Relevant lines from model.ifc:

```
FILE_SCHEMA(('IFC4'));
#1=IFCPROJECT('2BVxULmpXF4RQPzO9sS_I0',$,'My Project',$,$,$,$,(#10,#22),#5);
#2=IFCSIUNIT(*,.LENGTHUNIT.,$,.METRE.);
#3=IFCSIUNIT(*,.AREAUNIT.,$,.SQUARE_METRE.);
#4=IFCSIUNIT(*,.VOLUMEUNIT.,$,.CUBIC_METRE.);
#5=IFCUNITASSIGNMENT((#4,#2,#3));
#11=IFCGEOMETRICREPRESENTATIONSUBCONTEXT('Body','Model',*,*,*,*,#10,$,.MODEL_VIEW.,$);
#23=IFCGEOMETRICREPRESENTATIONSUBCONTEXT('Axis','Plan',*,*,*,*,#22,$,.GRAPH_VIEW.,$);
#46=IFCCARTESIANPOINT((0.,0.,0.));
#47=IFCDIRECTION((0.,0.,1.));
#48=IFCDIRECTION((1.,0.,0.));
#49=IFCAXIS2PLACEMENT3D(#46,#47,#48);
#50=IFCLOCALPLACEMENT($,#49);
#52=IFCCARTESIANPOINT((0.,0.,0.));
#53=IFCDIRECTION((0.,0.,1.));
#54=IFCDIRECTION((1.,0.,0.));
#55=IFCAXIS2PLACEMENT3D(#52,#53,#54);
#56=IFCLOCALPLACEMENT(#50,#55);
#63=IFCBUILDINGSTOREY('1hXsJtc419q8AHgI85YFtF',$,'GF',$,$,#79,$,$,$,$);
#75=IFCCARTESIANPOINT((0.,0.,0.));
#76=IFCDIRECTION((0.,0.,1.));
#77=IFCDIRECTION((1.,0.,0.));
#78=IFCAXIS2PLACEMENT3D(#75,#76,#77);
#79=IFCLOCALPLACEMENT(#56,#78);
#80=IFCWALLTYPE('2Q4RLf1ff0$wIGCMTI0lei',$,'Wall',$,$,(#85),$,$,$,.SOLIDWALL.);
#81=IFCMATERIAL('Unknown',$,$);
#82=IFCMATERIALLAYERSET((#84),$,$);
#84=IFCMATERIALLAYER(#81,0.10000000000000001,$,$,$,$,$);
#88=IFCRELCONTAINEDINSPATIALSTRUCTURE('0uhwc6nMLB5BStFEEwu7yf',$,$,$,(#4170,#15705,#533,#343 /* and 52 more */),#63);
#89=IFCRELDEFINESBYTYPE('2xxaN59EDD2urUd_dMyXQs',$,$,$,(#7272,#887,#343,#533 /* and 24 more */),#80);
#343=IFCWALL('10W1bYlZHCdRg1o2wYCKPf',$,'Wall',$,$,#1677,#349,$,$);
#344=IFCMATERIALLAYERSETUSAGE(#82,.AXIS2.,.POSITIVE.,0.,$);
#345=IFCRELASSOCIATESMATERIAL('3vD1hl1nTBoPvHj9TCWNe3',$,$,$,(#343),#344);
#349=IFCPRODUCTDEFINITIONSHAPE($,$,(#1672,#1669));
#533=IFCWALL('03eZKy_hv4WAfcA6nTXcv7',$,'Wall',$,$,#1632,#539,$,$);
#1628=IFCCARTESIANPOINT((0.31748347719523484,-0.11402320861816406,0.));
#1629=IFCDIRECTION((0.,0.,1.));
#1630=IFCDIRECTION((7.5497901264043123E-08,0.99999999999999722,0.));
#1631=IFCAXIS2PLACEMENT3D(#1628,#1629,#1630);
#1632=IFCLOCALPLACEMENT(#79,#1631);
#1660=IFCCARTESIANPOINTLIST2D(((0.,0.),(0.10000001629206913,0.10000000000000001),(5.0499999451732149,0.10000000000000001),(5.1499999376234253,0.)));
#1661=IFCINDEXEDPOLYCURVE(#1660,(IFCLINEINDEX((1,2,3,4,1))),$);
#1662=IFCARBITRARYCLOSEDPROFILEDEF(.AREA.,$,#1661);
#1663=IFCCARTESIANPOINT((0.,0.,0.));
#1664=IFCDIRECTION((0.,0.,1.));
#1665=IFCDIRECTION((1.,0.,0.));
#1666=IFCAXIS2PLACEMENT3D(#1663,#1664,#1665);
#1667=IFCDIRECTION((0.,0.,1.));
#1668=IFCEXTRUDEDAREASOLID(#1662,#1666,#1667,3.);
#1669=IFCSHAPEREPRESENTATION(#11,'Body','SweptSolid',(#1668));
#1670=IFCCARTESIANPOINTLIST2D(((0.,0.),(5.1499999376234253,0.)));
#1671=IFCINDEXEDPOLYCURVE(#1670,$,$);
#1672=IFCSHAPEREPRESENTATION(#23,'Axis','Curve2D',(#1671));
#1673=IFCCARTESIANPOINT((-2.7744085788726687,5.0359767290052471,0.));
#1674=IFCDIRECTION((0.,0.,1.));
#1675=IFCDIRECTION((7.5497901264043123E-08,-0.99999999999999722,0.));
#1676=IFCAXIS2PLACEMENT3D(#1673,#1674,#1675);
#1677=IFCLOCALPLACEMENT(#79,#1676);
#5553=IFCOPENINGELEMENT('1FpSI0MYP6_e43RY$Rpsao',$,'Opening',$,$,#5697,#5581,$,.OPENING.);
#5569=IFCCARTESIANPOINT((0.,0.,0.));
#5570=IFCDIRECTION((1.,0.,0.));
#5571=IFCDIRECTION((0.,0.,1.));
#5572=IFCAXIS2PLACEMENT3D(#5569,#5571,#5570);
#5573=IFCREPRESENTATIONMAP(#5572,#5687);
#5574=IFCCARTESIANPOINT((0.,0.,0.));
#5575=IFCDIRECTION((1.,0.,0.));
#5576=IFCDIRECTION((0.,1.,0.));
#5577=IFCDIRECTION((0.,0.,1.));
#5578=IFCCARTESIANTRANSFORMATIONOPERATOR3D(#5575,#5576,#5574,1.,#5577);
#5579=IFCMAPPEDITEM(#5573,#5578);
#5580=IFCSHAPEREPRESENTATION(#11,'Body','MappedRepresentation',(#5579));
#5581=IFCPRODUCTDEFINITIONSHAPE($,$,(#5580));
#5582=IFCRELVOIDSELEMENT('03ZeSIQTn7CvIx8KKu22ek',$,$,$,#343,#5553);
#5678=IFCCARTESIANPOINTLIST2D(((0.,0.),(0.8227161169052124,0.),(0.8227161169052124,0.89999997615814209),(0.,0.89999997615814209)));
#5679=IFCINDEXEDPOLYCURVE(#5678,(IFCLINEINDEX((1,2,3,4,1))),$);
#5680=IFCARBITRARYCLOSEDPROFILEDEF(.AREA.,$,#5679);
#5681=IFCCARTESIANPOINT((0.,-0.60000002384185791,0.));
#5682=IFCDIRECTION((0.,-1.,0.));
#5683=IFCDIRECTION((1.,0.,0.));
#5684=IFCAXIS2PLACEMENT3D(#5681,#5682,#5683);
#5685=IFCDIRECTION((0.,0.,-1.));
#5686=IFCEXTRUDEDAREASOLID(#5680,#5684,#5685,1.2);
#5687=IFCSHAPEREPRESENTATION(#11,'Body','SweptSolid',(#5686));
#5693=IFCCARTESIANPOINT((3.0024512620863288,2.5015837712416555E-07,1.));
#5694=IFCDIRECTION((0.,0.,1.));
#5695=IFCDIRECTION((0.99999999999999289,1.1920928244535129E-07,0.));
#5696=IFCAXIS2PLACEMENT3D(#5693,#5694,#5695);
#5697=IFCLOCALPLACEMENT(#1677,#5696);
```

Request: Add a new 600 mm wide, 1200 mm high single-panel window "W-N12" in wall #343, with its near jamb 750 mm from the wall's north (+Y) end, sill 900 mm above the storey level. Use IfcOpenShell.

```python
import numpy as np
import ifcopenshell
import ifcopenshell.api.feature
import ifcopenshell.api.geometry
import ifcopenshell.api.root
import ifcopenshell.api.spatial
import ifcopenshell.geom
import ifcopenshell.util.element
import ifcopenshell.util.placement
import ifcopenshell.util.representation
import ifcopenshell.util.shape
import ifcopenshell.util.unit

model = ifcopenshell.open("model.ifc")
unit_scale = ifcopenshell.util.unit.calculate_unit_scale(model)
settings = ifcopenshell.geom.settings()


def volume(element):
    """Net volume in cubic metres, openings subtracted."""
    shape = ifcopenshell.geom.create_shape(settings, element)
    return ifcopenshell.util.shape.get_volume(shape.geometry)


wall = model.by_guid("10W1bYlZHCdRg1o2wYCKPf")
storey = ifcopenshell.util.element.get_container(wall, ifc_class="IfcBuildingStorey")
context = ifcopenshell.util.representation.get_context(model, "Model", "Body", "MODEL_VIEW")
before = volume(wall)

width, height, from_end, sill = 0.6, 1.2, 0.75, 0.9  # metres

# The wall runs along its own X axis, and the end named is its -X end.
wall_shape = ifcopenshell.geom.create_shape(settings, wall)
x, y, z = ifcopenshell.util.shape.get_vertices(wall_shape.geometry).T
start = x.min() + from_end
face, thickness = float(y.min()), float(y.max() - y.min())
wall_matrix = ifcopenshell.util.placement.get_local_placement(wall.ObjectPlacement)
level = ifcopenshell.util.placement.get_local_placement(storey.ObjectPlacement)[2, 3]


def in_wall(x, y):
    """Placement at x, y metres in the wall's axes, at sill height."""
    matrix = wall_matrix.copy()
    matrix[:, 3] = wall_matrix @ np.array([x / unit_scale, y / unit_scale, 0.0, 1.0])
    matrix[2, 3] = level + sill / unit_scale
    return matrix


# Opening: a box that overshoots both wall faces by 50 mm.
opening = ifcopenshell.api.root.create_entity(model, ifc_class="IfcOpeningElement", predefined_type="OPENING")
box = ifcopenshell.api.geometry.add_wall_representation(
    model, context=context, length=width, height=height, thickness=thickness + 0.1
)
ifcopenshell.api.geometry.assign_representation(model, product=opening, representation=box)
ifcopenshell.api.geometry.edit_object_placement(model, product=opening, matrix=in_wall(start, face - 0.05), is_si=False)
ifcopenshell.api.feature.add_feature(model, feature=opening, element=wall)

window = ifcopenshell.api.root.create_entity(model, ifc_class="IfcWindow", name="W-N12", predefined_type="WINDOW")
window.OverallWidth, window.OverallHeight = width / unit_scale, height / unit_scale
window.PartitioningType = "SINGLE_PANEL"
body = ifcopenshell.api.geometry.add_window_representation(
    model,
    context=context,
    overall_width=window.OverallWidth,
    overall_height=window.OverallHeight,
    partition_type="SINGLE_PANEL",
)
ifcopenshell.api.geometry.assign_representation(model, product=window, representation=body)
ifcopenshell.api.spatial.assign_container(model, products=[window], relating_structure=storey)
ifcopenshell.api.feature.add_filling(model, opening=opening, element=window)

# Centre the window in the wall's thickness.
ifcopenshell.api.geometry.edit_object_placement(model, product=window, matrix=in_wall(start, face), is_si=False)
window_shape = ifcopenshell.geom.create_shape(settings, window)
depth = ifcopenshell.util.shape.get_vertices(window_shape.geometry)[:, 1]
offset = face + thickness / 2 - (depth.min() + depth.max()) / 2
ifcopenshell.api.geometry.edit_object_placement(model, product=window, matrix=in_wall(start, offset), is_si=False)

after = volume(wall)

print(f"wall volume {before:.3f} -> {after:.3f} m3")

model.write("model-out.ifc")
```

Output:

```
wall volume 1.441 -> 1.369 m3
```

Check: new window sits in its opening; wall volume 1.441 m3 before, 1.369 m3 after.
